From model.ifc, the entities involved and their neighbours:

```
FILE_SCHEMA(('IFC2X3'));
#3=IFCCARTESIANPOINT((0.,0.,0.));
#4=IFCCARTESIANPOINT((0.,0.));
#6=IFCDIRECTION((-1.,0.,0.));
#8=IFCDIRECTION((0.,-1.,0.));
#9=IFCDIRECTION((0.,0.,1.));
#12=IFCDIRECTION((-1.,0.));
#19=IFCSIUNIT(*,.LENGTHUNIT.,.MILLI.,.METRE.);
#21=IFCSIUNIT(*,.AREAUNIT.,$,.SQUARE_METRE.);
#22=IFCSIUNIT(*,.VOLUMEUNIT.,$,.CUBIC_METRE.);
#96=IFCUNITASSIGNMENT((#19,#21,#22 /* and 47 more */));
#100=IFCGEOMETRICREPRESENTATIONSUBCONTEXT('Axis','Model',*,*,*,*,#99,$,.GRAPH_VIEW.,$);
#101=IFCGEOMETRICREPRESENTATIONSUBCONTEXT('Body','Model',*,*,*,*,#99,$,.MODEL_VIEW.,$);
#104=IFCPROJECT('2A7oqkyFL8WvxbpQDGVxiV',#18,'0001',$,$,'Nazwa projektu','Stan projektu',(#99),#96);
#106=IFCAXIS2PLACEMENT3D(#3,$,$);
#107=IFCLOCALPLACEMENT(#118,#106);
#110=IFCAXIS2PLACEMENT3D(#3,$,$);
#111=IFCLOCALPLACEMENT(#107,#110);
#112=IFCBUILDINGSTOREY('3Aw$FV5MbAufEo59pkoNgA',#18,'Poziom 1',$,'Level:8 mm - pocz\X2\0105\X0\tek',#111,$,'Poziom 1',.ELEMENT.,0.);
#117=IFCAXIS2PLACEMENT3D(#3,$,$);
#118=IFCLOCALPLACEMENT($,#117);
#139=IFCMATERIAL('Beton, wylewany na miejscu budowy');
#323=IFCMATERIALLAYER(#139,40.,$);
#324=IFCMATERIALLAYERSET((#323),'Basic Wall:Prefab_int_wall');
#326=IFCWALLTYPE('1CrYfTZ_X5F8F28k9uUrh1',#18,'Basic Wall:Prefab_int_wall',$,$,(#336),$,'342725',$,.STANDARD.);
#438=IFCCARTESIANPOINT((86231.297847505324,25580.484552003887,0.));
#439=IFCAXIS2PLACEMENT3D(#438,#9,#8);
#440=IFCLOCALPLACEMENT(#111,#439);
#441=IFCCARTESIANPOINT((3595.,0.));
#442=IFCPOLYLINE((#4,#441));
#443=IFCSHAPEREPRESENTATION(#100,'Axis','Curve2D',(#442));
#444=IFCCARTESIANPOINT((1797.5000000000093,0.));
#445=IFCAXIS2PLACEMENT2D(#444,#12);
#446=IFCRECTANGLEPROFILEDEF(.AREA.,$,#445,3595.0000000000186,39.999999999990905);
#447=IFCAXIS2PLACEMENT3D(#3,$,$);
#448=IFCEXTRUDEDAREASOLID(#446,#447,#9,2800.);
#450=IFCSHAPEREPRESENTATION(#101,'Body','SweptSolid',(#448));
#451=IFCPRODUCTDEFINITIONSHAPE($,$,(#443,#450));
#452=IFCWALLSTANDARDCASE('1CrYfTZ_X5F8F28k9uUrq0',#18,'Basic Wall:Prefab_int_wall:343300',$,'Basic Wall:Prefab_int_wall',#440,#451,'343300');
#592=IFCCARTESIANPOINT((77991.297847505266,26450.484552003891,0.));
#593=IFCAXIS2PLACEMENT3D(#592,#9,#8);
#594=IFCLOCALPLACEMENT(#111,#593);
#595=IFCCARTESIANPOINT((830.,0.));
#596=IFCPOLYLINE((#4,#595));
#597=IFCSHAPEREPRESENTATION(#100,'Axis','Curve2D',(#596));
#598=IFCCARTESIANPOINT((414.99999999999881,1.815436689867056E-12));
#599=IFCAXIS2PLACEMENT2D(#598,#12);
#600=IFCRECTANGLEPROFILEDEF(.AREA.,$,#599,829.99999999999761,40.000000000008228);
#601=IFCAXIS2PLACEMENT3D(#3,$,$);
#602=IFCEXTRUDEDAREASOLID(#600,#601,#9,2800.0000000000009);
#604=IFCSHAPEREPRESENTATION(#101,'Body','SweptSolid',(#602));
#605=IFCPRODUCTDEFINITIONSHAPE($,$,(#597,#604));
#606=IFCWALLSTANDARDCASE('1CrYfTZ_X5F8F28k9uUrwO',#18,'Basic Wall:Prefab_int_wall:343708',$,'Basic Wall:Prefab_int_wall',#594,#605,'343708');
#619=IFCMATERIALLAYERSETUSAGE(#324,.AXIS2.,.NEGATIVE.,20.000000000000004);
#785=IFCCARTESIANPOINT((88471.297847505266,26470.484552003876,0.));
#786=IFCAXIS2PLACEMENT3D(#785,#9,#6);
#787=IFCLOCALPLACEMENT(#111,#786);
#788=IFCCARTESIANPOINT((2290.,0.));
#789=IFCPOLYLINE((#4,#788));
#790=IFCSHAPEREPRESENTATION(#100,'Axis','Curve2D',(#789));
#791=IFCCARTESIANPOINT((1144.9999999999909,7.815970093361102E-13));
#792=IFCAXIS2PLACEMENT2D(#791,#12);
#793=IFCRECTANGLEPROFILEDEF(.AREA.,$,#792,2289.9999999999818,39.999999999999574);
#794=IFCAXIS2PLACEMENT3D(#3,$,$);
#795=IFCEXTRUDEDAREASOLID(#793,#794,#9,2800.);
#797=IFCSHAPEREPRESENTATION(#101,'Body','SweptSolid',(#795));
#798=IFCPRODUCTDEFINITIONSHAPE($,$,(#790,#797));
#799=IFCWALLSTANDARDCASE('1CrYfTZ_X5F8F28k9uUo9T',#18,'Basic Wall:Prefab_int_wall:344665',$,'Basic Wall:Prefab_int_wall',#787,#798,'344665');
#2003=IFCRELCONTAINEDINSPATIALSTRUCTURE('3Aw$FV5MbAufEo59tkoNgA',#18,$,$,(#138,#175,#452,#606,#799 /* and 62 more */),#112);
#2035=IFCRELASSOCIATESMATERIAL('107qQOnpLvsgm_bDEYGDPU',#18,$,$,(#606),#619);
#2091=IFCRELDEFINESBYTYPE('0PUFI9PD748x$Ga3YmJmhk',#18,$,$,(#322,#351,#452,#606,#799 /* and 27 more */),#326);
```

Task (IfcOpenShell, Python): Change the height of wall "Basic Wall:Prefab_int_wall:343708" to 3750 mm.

```python
import ifcopenshell
import ifcopenshell.geom
import ifcopenshell.util.representation
import ifcopenshell.util.shape
import ifcopenshell.util.unit

model = ifcopenshell.open("model.ifc")
unit_scale = ifcopenshell.util.unit.calculate_unit_scale(model)
settings = ifcopenshell.geom.settings()


def volume(element):
    """Net volume in cubic metres, openings subtracted."""
    shape = ifcopenshell.geom.create_shape(settings, element)
    return ifcopenshell.util.shape.get_volume(shape.geometry)


wall = model.by_id(606)
before = volume(wall)

body = ifcopenshell.util.representation.get_representation(wall, "Model", "Body")
solid = body.Items[0]
old_height = solid.Depth
solid.Depth = 3.75 / unit_scale
after = volume(wall)

print(f"height {old_height:g} -> {solid.Depth:g}, volume {before:.3f} -> {after:.3f} m3")

model.write("model_rev.ifc")
```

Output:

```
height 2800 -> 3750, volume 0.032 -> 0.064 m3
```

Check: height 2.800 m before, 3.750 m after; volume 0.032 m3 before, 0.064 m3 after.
